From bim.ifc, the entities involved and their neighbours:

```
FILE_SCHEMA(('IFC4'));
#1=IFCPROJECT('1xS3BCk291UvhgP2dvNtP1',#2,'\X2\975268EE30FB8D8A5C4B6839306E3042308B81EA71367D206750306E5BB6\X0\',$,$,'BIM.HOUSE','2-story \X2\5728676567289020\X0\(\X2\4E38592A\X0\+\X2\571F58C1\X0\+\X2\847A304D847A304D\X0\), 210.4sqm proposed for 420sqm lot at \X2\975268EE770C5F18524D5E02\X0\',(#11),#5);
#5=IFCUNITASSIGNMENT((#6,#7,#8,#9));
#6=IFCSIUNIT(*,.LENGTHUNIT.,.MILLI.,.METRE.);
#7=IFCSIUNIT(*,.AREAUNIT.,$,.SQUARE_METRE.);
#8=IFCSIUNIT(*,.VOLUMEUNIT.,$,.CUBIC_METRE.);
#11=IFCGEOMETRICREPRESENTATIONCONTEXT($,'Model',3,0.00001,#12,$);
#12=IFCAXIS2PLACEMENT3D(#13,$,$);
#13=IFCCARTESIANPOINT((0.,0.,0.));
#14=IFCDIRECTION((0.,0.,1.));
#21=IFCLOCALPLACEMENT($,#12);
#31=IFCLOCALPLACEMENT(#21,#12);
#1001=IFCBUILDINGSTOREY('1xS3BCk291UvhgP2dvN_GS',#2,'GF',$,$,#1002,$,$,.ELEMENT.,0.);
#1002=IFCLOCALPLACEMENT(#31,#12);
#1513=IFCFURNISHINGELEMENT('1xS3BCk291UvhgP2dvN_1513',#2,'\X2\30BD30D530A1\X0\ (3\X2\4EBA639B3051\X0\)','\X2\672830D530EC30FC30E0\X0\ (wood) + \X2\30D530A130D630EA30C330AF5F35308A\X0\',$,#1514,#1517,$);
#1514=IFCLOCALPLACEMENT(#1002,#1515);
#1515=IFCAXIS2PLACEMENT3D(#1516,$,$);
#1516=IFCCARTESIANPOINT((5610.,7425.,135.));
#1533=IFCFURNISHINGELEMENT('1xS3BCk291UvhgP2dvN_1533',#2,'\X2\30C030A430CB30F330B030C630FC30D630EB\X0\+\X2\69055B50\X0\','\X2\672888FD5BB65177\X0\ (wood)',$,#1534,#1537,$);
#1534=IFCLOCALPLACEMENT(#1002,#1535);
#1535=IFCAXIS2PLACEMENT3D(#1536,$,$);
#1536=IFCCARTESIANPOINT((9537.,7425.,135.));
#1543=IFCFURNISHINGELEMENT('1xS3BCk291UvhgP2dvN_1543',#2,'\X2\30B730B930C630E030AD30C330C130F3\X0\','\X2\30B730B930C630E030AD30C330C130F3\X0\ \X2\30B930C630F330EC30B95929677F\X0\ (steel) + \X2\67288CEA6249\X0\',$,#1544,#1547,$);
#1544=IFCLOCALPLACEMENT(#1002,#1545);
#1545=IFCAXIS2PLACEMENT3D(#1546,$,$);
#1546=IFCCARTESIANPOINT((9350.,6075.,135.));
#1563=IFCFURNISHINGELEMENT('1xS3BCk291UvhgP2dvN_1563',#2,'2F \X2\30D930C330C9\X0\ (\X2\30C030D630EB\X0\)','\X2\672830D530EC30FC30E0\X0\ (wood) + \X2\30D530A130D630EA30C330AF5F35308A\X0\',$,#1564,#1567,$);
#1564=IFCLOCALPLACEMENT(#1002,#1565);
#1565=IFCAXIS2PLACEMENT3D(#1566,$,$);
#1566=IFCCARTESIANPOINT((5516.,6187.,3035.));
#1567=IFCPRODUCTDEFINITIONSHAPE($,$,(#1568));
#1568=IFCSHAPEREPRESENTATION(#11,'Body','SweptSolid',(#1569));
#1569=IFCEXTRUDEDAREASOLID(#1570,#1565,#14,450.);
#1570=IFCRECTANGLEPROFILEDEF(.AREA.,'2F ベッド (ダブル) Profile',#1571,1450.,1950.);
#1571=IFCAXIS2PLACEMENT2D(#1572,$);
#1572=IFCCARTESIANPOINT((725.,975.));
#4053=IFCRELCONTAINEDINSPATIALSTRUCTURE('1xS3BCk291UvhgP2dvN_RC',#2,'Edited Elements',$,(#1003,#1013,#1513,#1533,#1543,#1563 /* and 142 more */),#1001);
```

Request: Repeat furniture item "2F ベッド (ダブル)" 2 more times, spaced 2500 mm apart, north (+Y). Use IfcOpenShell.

```python
import numpy as np
import ifcopenshell
import ifcopenshell.api.geometry
import ifcopenshell.api.root
import ifcopenshell.util.element
import ifcopenshell.util.placement
import ifcopenshell.util.unit

model = ifcopenshell.open("bim.ifc")
unit_scale = ifcopenshell.util.unit.calculate_unit_scale(model)


def reuse_history(source, copy):
    """copy_class also copies each property set's owner history, people and application; keep the originals."""
    for rel in copy.IsDefinedBy:
        if rel.is_a("IfcRelDefinesByProperties") and (history := rel.RelatingPropertyDefinition.OwnerHistory):
            rel.RelatingPropertyDefinition.OwnerHistory = source.OwnerHistory
            ifcopenshell.util.element.remove_deep2(model, history)


source = model.by_guid("1xS3BCk291UvhgP2dvN_1563")
base = ifcopenshell.util.placement.get_local_placement(source.ObjectPlacement)
step = np.array([0.0, 1.0, 0.0]) * 2.5 / unit_scale

for i in range(1, 3):
    copy = ifcopenshell.api.root.copy_class(model, product=source)
    copy.Representation = ifcopenshell.util.element.copy_deep(
        model, source.Representation, exclude=["IfcGeometricRepresentationContext", "IfcRepresentationMap"]
    )
    reuse_history(source, copy)
    matrix = base.copy()
    matrix[:3, 3] += i * step
    print("added at", matrix[:3, 3].round(3) + 0.0)
    ifcopenshell.api.geometry.edit_object_placement(model, product=copy, matrix=matrix, is_si=False)

model.write("bim-out.ifc")
```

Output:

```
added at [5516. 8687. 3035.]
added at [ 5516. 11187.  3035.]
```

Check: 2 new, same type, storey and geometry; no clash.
